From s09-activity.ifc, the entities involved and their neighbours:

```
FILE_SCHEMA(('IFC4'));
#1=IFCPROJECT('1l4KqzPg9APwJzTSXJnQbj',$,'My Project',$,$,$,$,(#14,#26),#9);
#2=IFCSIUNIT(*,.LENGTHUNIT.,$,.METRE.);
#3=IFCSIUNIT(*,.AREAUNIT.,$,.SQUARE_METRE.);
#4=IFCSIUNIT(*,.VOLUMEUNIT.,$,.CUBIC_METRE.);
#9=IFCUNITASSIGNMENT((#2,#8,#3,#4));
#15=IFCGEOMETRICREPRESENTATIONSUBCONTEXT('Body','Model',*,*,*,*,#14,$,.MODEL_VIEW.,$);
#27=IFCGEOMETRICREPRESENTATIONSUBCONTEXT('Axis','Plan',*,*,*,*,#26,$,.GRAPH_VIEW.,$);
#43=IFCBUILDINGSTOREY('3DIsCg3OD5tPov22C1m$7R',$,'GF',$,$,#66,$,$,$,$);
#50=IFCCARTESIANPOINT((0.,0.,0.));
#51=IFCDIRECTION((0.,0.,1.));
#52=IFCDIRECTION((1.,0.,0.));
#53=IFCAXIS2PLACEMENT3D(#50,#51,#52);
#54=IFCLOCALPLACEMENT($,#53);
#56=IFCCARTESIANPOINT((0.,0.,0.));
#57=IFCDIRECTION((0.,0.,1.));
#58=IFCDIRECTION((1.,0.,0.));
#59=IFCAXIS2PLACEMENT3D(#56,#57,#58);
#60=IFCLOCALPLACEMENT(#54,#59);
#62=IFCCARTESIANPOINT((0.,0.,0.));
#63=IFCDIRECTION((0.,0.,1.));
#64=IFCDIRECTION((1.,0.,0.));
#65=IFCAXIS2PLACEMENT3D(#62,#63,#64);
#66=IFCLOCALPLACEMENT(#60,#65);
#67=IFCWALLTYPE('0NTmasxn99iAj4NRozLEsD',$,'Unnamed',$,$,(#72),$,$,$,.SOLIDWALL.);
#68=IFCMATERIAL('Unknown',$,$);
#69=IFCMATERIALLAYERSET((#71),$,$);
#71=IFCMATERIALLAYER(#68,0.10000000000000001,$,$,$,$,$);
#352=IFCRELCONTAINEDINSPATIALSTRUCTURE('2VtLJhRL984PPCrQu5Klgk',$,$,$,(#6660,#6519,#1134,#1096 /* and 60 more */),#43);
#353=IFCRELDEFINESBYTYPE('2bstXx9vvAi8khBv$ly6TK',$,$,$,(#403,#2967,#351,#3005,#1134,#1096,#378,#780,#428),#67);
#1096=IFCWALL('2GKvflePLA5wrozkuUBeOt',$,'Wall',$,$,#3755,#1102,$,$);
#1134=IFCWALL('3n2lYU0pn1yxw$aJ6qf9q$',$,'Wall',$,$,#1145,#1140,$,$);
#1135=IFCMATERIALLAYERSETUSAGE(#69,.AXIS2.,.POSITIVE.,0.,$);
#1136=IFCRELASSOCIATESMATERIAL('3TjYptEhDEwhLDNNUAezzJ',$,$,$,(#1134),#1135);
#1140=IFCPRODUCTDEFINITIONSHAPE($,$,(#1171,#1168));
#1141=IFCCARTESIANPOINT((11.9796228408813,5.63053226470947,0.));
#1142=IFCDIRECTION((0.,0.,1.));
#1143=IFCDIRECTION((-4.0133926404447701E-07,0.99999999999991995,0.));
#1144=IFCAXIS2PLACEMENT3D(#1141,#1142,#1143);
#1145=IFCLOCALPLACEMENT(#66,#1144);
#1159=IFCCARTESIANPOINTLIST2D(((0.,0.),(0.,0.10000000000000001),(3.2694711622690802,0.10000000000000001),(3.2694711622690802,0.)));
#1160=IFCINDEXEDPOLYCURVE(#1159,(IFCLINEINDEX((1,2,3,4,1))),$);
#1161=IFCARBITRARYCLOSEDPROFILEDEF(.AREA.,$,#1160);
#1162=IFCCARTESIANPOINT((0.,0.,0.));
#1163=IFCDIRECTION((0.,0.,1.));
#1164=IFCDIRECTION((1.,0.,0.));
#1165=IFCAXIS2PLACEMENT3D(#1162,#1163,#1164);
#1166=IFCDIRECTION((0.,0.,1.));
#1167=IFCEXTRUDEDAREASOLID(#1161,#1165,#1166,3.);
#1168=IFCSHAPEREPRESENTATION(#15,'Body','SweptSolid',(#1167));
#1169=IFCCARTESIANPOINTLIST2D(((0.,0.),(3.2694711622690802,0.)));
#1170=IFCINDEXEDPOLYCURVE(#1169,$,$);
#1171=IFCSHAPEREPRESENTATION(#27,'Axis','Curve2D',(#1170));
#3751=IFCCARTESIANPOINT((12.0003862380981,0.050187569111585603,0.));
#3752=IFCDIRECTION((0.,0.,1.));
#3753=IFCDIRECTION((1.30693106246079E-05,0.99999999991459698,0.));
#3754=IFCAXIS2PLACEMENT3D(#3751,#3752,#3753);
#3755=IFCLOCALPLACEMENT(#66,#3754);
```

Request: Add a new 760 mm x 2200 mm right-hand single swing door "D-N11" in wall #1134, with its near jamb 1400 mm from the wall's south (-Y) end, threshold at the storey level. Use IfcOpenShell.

```python
import numpy as np
import ifcopenshell
import ifcopenshell.api.feature
import ifcopenshell.api.geometry
import ifcopenshell.api.root
import ifcopenshell.api.spatial
import ifcopenshell.geom
import ifcopenshell.util.element
import ifcopenshell.util.placement
import ifcopenshell.util.representation
import ifcopenshell.util.shape
import ifcopenshell.util.unit

model = ifcopenshell.open("s09-activity.ifc")
unit_scale = ifcopenshell.util.unit.calculate_unit_scale(model)
settings = ifcopenshell.geom.settings()


def volume(element):
    """Net volume in cubic metres, openings subtracted."""
    shape = ifcopenshell.geom.create_shape(settings, element)
    return ifcopenshell.util.shape.get_volume(shape.geometry)


wall = model.by_guid("3n2lYU0pn1yxw$aJ6qf9q$")
storey = ifcopenshell.util.element.get_container(wall, ifc_class="IfcBuildingStorey")
context = ifcopenshell.util.representation.get_context(model, "Model", "Body", "MODEL_VIEW")
before = volume(wall)

width, height, from_end, sill = 0.76, 2.2, 1.4, 0.0  # metres

# The wall runs along its own X axis, and the end named is its -X end.
wall_shape = ifcopenshell.geom.create_shape(settings, wall)
x, y, z = ifcopenshell.util.shape.get_vertices(wall_shape.geometry).T
start = x.min() + from_end
face, thickness = float(y.min()), float(y.max() - y.min())
wall_matrix = ifcopenshell.util.placement.get_local_placement(wall.ObjectPlacement)
level = ifcopenshell.util.placement.get_local_placement(storey.ObjectPlacement)[2, 3]


def in_wall(x, y):
    """Placement at x, y metres in the wall's axes, at sill height."""
    matrix = wall_matrix.copy()
    matrix[:, 3] = wall_matrix @ np.array([x / unit_scale, y / unit_scale, 0.0, 1.0])
    matrix[2, 3] = level + sill / unit_scale
    return matrix


# Opening: a box that overshoots both wall faces by 50 mm.
opening = ifcopenshell.api.root.create_entity(model, ifc_class="IfcOpeningElement", predefined_type="OPENING")
box = ifcopenshell.api.geometry.add_wall_representation(
    model, context=context, length=width, height=height, thickness=thickness + 0.1
)
ifcopenshell.api.geometry.assign_representation(model, product=opening, representation=box)
ifcopenshell.api.geometry.edit_object_placement(model, product=opening, matrix=in_wall(start, face - 0.05), is_si=False)
ifcopenshell.api.feature.add_feature(model, feature=opening, element=wall)

door = ifcopenshell.api.root.create_entity(model, ifc_class="IfcDoor", name="D-N11", predefined_type="DOOR")
door.OverallWidth, door.OverallHeight = width / unit_scale, height / unit_scale
door.OperationType = "SINGLE_SWING_RIGHT"
body = ifcopenshell.api.geometry.add_door_representation(
    model,
    context=context,
    overall_width=door.OverallWidth,
    overall_height=door.OverallHeight,
    operation_type="SINGLE_SWING_RIGHT",
    lining_properties={"LiningDepth": thickness / unit_scale, "ThresholdDepth": thickness / unit_scale},
)
ifcopenshell.api.geometry.assign_representation(model, product=door, representation=body)
ifcopenshell.api.spatial.assign_container(model, products=[door], relating_structure=storey)
ifcopenshell.api.feature.add_filling(model, opening=opening, element=door)

# The lining spans the wall, so the door starts at the wall face.
ifcopenshell.api.geometry.edit_object_placement(model, product=door, matrix=in_wall(start, face), is_si=False)

after = volume(wall)

print(f"wall volume {before:.3f} -> {after:.3f} m3")

model.write("s09-activity_updated.ifc")
```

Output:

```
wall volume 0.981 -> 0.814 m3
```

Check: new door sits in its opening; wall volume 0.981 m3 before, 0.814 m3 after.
